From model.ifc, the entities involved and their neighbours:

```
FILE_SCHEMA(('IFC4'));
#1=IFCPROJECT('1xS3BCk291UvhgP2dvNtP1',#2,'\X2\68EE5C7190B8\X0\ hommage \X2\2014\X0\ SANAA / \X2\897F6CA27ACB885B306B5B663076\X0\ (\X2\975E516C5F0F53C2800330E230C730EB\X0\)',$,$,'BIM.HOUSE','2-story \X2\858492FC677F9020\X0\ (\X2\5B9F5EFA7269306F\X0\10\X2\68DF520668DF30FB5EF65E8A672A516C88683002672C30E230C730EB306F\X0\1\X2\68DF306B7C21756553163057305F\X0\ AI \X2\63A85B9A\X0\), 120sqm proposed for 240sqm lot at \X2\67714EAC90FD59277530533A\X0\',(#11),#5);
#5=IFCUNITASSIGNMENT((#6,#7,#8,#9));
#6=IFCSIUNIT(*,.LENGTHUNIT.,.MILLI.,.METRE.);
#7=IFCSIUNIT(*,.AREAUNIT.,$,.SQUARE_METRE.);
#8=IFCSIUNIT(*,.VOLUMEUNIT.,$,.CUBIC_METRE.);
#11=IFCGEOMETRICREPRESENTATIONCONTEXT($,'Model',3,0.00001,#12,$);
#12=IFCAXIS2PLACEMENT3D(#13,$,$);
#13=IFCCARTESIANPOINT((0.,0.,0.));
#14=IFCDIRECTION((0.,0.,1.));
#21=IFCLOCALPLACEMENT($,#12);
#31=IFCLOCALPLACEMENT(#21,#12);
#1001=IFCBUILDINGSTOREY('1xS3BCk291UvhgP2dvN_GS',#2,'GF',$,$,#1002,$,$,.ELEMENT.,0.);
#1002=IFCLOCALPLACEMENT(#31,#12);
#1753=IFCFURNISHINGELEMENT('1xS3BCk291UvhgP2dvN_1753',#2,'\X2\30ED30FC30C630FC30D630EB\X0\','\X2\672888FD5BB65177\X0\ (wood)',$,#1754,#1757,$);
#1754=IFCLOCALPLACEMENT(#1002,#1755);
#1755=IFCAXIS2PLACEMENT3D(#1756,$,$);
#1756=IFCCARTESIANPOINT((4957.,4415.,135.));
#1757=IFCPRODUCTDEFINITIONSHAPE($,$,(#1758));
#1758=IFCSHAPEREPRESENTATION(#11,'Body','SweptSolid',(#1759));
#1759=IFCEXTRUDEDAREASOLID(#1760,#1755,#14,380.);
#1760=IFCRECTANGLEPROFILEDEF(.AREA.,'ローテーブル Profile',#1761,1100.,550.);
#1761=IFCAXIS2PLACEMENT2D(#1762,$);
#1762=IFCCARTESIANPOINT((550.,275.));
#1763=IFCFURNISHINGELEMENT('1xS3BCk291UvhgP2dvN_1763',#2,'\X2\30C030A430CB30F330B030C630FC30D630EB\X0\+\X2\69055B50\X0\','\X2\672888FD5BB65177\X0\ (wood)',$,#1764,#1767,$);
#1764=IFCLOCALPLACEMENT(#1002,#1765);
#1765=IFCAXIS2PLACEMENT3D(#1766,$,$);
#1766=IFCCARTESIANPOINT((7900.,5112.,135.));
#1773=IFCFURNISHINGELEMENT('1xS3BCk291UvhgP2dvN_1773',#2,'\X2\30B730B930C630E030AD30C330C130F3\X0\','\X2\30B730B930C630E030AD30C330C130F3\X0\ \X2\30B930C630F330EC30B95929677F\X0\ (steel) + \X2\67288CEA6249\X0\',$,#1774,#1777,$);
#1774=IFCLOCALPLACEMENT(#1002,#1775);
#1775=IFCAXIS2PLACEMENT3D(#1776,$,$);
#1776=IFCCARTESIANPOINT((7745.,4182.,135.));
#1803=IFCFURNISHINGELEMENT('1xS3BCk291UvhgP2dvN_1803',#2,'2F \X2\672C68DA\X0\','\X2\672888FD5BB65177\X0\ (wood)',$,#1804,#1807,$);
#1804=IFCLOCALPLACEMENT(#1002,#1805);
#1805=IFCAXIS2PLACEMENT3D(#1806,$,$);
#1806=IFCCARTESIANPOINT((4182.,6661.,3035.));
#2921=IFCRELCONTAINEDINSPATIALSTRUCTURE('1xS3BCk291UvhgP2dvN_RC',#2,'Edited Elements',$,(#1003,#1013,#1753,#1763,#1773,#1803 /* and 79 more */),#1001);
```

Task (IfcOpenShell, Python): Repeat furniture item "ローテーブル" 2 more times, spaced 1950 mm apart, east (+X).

```python
import numpy as np
import ifcopenshell
import ifcopenshell.api.geometry
import ifcopenshell.api.root
import ifcopenshell.util.element
import ifcopenshell.util.placement
import ifcopenshell.util.unit

model = ifcopenshell.open("model.ifc")
unit_scale = ifcopenshell.util.unit.calculate_unit_scale(model)


def reuse_history(source, copy):
    """copy_class also copies each property set's owner history, people and application; keep the originals."""
    for rel in copy.IsDefinedBy:
        if rel.is_a("IfcRelDefinesByProperties") and (history := rel.RelatingPropertyDefinition.OwnerHistory):
            rel.RelatingPropertyDefinition.OwnerHistory = source.OwnerHistory
            ifcopenshell.util.element.remove_deep2(model, history)


source = model.by_guid("1xS3BCk291UvhgP2dvN_1753")
base = ifcopenshell.util.placement.get_local_placement(source.ObjectPlacement)
step = np.array([1.0, 0.0, 0.0]) * 1.95 / unit_scale

for i in range(1, 3):
    copy = ifcopenshell.api.root.copy_class(model, product=source)
    copy.Representation = ifcopenshell.util.element.copy_deep(
        model, source.Representation, exclude=["IfcGeometricRepresentationContext", "IfcRepresentationMap"]
    )
    reuse_history(source, copy)
    matrix = base.copy()
    matrix[:3, 3] += i * step
    print("added at", matrix[:3, 3].round(3) + 0.0)
    ifcopenshell.api.geometry.edit_object_placement(model, product=copy, matrix=matrix, is_si=False)

model.write("model_edited.ifc")
```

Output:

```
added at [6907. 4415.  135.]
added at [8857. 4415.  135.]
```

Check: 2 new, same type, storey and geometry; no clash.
